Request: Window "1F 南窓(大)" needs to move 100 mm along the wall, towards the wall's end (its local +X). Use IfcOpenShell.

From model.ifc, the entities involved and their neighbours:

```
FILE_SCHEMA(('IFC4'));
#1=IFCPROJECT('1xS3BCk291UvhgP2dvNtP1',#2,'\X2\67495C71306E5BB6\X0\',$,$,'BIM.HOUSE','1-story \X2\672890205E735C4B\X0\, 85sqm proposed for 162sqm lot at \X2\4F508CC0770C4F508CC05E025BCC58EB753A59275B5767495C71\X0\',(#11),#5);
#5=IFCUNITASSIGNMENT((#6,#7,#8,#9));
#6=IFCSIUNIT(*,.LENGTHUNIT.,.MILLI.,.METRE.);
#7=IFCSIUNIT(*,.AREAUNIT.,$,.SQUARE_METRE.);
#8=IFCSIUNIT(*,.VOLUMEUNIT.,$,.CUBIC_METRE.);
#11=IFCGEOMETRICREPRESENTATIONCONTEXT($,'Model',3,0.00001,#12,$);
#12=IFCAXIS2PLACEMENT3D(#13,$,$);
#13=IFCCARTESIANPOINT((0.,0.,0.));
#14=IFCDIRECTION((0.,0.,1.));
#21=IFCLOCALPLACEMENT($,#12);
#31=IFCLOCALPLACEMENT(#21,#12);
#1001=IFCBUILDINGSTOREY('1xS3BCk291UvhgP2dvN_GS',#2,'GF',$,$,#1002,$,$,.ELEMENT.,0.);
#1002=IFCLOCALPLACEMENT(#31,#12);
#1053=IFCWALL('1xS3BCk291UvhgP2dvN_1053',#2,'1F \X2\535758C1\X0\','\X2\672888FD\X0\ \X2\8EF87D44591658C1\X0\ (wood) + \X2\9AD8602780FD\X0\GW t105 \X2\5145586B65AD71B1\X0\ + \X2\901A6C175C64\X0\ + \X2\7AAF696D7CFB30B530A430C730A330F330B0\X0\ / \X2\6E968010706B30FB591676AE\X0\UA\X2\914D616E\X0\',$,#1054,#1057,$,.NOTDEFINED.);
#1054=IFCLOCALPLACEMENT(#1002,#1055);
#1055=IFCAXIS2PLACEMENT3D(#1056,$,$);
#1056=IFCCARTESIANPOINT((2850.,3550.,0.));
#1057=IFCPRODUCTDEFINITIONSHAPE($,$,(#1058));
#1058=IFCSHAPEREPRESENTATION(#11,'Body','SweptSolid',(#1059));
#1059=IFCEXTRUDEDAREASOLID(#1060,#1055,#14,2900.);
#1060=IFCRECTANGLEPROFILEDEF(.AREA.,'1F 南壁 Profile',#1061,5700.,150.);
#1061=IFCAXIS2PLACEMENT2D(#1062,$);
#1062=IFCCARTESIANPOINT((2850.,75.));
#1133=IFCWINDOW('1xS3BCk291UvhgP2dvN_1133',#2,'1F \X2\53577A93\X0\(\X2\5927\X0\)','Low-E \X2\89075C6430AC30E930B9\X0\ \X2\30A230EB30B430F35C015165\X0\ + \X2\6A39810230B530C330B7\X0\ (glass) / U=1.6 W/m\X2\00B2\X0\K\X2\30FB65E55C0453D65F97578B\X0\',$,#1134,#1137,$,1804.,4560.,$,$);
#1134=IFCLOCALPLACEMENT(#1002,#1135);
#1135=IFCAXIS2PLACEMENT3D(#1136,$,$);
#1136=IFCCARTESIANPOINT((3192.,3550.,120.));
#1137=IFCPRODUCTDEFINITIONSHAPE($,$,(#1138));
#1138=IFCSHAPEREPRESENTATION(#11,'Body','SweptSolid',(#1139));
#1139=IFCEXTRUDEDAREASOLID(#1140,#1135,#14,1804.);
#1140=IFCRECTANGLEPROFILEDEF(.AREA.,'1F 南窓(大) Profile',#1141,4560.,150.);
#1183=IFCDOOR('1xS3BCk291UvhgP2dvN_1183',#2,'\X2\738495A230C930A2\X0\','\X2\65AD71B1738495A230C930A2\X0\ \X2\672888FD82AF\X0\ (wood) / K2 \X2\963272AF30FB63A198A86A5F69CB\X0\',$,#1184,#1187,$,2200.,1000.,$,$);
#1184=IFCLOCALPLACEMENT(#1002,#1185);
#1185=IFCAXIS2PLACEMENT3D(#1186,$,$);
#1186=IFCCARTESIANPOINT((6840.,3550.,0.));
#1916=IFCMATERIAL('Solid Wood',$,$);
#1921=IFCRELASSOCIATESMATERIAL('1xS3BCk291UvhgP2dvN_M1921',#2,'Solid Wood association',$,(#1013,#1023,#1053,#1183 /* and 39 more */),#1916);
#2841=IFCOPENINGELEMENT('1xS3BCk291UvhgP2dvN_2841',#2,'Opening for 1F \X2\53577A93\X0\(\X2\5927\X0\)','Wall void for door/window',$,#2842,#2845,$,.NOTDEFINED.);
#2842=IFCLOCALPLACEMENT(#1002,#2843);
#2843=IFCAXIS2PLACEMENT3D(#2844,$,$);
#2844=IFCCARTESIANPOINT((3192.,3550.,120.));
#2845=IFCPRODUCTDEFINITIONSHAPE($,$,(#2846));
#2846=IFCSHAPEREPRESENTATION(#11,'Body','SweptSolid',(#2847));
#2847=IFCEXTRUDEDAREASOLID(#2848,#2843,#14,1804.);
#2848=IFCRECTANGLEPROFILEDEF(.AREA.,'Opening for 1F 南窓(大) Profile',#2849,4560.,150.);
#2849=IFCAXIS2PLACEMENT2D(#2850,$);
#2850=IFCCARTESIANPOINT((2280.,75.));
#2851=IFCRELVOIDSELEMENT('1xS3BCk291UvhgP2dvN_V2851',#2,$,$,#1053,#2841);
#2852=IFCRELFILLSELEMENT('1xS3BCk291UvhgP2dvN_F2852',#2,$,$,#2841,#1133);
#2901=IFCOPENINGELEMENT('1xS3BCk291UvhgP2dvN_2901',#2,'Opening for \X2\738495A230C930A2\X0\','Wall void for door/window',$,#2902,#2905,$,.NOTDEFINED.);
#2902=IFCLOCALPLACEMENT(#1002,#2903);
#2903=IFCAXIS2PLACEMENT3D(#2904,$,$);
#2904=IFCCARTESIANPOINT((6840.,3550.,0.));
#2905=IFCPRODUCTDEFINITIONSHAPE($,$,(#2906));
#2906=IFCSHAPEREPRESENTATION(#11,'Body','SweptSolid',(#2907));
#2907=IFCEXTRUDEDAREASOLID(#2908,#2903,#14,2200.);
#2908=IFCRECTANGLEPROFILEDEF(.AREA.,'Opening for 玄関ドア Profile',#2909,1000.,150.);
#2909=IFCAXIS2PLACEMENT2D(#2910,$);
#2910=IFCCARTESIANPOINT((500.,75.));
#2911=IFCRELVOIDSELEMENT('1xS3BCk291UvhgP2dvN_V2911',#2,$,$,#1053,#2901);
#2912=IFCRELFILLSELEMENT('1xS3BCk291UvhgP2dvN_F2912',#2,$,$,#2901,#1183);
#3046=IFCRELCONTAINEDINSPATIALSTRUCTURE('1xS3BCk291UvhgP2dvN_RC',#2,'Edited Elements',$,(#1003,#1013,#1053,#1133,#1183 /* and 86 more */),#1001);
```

```python
import ifcopenshell
import ifcopenshell.api.geometry
import ifcopenshell.util.placement
import ifcopenshell.util.unit

model = ifcopenshell.open("model.ifc")
unit_scale = ifcopenshell.util.unit.calculate_unit_scale(model)

window = model.by_guid("1xS3BCk291UvhgP2dvN_1133")
opening = window.FillsVoids[0].RelatingOpeningElement
wall = opening.VoidsElements[0].RelatingBuildingElement

wall_matrix = ifcopenshell.util.placement.get_local_placement(wall.ObjectPlacement)
shift = wall_matrix[:3, 0] * 0.1 / unit_scale
before = ifcopenshell.util.placement.get_local_placement(window.ObjectPlacement)[:3, 3].copy()

# The window is not placed relative to its opening, so move both.
for product in (opening, window):
    matrix = ifcopenshell.util.placement.get_local_placement(product.ObjectPlacement)
    matrix[:3, 3] += shift
    ifcopenshell.api.geometry.edit_object_placement(model, product=product, matrix=matrix, is_si=False)

after = ifcopenshell.util.placement.get_local_placement(window.ObjectPlacement)[:3, 3]
print("window moved by", (after - before).round(3) + 0.0)

model.write("model_v2.ifc")
```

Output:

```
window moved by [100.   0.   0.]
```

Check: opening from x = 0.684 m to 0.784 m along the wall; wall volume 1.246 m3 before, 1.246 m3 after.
